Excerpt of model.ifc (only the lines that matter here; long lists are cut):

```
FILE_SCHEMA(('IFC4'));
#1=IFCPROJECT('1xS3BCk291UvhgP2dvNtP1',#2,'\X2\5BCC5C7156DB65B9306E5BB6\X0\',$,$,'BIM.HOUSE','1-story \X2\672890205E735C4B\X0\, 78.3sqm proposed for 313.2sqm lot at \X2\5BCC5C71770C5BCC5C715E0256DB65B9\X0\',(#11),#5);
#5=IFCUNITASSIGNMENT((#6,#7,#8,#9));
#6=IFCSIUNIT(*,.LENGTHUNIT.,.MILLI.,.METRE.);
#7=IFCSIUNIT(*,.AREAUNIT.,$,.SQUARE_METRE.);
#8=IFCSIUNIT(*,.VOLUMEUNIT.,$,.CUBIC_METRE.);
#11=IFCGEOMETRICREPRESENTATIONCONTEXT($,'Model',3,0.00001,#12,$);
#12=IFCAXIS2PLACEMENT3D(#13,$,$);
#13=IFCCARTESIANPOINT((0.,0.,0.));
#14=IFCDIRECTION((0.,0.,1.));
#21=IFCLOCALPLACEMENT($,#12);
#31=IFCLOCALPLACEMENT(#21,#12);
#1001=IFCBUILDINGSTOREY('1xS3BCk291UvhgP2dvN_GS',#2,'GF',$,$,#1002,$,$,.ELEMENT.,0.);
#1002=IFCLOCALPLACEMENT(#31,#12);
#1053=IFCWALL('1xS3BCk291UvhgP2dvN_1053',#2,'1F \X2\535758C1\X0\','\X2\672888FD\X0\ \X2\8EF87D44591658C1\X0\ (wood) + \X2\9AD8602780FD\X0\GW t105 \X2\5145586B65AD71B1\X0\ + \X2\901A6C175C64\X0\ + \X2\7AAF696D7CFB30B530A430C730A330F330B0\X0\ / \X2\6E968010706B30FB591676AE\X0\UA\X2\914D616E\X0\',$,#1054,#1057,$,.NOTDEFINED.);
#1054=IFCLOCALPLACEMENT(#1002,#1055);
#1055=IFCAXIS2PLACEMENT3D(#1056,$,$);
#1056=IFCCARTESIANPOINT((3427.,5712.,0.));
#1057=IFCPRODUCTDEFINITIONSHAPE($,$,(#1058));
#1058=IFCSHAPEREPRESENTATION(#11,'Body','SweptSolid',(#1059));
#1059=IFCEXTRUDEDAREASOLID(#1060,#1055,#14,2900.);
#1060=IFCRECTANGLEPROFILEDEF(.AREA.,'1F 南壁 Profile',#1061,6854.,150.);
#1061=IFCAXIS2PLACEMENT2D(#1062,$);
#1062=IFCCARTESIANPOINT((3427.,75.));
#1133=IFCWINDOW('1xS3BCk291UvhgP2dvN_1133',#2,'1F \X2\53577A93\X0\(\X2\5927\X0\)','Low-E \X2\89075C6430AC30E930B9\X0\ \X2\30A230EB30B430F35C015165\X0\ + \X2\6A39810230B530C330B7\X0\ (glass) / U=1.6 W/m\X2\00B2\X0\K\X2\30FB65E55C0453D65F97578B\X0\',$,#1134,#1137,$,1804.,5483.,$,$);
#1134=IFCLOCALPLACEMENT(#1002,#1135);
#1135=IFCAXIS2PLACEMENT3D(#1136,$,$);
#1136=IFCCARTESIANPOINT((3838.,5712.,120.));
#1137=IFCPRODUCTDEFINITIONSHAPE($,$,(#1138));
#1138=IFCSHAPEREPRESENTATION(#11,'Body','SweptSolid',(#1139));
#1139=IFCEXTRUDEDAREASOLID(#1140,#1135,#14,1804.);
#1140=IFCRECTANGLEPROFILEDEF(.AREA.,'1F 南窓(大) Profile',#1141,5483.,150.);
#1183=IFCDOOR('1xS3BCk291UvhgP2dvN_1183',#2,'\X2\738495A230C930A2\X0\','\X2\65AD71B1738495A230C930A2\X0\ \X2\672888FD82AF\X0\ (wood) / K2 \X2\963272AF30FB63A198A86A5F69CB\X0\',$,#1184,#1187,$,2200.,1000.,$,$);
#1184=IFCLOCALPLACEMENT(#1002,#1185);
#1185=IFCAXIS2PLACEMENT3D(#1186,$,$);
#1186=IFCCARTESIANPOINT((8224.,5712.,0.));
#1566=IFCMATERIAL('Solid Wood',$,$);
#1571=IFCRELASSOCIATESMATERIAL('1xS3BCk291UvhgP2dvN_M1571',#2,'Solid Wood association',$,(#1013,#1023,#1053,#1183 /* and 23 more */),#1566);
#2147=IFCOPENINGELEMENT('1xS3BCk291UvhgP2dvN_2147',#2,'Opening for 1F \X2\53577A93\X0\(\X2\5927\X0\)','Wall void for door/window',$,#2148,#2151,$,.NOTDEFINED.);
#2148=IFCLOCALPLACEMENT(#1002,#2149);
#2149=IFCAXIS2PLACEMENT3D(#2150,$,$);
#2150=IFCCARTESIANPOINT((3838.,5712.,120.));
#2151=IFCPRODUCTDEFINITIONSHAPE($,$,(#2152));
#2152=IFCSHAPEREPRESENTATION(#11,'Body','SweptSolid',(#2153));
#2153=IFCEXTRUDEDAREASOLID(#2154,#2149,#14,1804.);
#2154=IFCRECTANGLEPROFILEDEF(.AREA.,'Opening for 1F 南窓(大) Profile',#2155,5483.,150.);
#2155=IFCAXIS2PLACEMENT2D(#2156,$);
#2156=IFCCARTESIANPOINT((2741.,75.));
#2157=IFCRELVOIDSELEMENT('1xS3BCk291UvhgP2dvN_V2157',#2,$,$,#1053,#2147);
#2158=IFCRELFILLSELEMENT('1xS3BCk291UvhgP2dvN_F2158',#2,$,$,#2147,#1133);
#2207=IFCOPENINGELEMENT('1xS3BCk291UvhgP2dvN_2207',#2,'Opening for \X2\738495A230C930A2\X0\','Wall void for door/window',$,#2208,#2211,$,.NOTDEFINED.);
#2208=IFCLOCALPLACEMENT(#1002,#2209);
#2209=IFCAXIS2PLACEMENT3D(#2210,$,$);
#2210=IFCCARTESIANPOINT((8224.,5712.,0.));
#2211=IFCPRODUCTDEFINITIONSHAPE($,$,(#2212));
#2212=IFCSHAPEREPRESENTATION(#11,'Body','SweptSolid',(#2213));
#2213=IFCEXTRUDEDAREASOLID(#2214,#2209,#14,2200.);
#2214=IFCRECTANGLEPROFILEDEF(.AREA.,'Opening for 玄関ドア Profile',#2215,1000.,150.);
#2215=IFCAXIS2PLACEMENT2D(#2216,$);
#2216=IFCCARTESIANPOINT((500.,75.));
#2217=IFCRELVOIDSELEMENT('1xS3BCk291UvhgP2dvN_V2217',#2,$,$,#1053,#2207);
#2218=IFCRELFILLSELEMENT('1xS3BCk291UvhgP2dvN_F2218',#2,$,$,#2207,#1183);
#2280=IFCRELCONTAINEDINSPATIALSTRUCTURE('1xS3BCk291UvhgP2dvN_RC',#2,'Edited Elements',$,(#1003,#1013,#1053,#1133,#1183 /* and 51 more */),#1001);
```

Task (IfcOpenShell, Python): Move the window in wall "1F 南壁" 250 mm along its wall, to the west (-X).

```python
import ifcopenshell
import ifcopenshell.api.geometry
import ifcopenshell.util.placement
import ifcopenshell.util.unit

model = ifcopenshell.open("model.ifc")
unit_scale = ifcopenshell.util.unit.calculate_unit_scale(model)

window = model.by_guid("1xS3BCk291UvhgP2dvN_1133")
opening = window.FillsVoids[0].RelatingOpeningElement
wall = opening.VoidsElements[0].RelatingBuildingElement

wall_matrix = ifcopenshell.util.placement.get_local_placement(wall.ObjectPlacement)
shift = wall_matrix[:3, 0] * -0.25 / unit_scale
before = ifcopenshell.util.placement.get_local_placement(window.ObjectPlacement)[:3, 3].copy()

# The window is not placed relative to its opening, so move both.
for product in (opening, window):
    matrix = ifcopenshell.util.placement.get_local_placement(product.ObjectPlacement)
    matrix[:3, 3] += shift
    ifcopenshell.api.geometry.edit_object_placement(model, product=product, matrix=matrix, is_si=False)

after = ifcopenshell.util.placement.get_local_placement(window.ObjectPlacement)[:3, 3]
print("window moved by", (after - before).round(3) + 0.0)

model.write("model_updated.ifc")
```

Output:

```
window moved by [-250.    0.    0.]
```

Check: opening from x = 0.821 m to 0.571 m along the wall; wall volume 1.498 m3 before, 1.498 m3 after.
